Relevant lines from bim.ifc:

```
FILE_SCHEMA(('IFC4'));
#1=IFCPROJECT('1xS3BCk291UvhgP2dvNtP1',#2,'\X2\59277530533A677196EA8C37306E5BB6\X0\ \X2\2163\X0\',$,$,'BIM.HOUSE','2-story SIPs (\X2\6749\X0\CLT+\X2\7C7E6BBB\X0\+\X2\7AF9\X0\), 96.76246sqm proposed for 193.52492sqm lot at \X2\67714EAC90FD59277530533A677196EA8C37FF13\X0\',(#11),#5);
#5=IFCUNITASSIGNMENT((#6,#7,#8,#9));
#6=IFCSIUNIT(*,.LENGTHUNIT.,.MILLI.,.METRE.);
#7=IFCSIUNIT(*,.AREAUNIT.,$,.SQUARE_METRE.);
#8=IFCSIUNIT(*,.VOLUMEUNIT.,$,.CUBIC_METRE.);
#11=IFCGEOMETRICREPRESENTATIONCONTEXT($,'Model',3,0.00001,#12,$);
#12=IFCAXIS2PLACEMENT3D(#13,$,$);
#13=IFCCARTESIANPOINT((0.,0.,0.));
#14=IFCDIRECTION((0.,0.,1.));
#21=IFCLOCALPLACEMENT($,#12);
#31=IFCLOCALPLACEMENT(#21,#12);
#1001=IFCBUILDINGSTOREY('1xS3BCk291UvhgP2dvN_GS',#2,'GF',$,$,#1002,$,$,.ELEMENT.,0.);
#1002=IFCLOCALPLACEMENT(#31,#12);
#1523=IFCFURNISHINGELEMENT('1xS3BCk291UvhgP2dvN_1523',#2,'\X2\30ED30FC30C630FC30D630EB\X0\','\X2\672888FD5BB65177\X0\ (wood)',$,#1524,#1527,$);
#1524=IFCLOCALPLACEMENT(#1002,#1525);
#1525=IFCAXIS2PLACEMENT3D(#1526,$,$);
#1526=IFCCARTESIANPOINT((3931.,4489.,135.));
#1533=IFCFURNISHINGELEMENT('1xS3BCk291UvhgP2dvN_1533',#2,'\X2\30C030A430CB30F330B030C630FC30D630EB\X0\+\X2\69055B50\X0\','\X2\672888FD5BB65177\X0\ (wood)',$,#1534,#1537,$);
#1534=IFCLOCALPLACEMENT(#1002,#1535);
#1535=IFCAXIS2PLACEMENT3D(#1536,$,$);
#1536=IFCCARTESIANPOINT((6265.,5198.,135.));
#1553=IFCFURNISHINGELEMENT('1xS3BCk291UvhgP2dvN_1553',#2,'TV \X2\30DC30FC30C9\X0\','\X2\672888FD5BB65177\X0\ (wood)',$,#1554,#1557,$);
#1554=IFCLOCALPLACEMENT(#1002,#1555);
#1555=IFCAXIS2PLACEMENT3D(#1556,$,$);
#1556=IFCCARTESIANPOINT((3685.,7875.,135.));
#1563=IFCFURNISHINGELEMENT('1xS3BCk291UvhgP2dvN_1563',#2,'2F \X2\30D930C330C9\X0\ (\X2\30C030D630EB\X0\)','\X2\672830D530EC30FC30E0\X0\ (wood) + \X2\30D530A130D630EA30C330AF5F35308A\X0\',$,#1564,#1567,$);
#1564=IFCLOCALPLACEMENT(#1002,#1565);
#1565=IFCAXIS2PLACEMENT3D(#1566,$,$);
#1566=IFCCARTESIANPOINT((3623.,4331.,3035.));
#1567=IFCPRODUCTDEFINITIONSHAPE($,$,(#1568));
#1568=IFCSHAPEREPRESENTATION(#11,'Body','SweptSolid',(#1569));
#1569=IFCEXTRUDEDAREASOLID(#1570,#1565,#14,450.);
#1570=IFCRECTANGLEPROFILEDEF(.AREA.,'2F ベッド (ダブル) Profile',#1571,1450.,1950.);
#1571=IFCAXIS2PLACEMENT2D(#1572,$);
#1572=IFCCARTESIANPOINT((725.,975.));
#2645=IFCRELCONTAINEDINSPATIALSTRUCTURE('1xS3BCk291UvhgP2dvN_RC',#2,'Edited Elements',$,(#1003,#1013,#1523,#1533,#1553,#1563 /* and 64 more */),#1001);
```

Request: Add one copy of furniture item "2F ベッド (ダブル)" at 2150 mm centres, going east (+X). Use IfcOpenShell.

```python
import numpy as np
import ifcopenshell
import ifcopenshell.api.geometry
import ifcopenshell.api.root
import ifcopenshell.util.element
import ifcopenshell.util.placement
import ifcopenshell.util.unit

model = ifcopenshell.open("bim.ifc")
unit_scale = ifcopenshell.util.unit.calculate_unit_scale(model)


def reuse_history(source, copy):
    """copy_class also copies each property set's owner history, people and application; keep the originals."""
    for rel in copy.IsDefinedBy:
        if rel.is_a("IfcRelDefinesByProperties") and (history := rel.RelatingPropertyDefinition.OwnerHistory):
            rel.RelatingPropertyDefinition.OwnerHistory = source.OwnerHistory
            ifcopenshell.util.element.remove_deep2(model, history)


source = model.by_guid("1xS3BCk291UvhgP2dvN_1563")
base = ifcopenshell.util.placement.get_local_placement(source.ObjectPlacement)
step = np.array([1.0, 0.0, 0.0]) * 2.15 / unit_scale

for i in range(1, 2):
    copy = ifcopenshell.api.root.copy_class(model, product=source)
    copy.Representation = ifcopenshell.util.element.copy_deep(
        model, source.Representation, exclude=["IfcGeometricRepresentationContext", "IfcRepresentationMap"]
    )
    reuse_history(source, copy)
    matrix = base.copy()
    matrix[:3, 3] += i * step
    print("added at", matrix[:3, 3].round(3) + 0.0)
    ifcopenshell.api.geometry.edit_object_placement(model, product=copy, matrix=matrix, is_si=False)

model.write("bim_rev.ifc")
```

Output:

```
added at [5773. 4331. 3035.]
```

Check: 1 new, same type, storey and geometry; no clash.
